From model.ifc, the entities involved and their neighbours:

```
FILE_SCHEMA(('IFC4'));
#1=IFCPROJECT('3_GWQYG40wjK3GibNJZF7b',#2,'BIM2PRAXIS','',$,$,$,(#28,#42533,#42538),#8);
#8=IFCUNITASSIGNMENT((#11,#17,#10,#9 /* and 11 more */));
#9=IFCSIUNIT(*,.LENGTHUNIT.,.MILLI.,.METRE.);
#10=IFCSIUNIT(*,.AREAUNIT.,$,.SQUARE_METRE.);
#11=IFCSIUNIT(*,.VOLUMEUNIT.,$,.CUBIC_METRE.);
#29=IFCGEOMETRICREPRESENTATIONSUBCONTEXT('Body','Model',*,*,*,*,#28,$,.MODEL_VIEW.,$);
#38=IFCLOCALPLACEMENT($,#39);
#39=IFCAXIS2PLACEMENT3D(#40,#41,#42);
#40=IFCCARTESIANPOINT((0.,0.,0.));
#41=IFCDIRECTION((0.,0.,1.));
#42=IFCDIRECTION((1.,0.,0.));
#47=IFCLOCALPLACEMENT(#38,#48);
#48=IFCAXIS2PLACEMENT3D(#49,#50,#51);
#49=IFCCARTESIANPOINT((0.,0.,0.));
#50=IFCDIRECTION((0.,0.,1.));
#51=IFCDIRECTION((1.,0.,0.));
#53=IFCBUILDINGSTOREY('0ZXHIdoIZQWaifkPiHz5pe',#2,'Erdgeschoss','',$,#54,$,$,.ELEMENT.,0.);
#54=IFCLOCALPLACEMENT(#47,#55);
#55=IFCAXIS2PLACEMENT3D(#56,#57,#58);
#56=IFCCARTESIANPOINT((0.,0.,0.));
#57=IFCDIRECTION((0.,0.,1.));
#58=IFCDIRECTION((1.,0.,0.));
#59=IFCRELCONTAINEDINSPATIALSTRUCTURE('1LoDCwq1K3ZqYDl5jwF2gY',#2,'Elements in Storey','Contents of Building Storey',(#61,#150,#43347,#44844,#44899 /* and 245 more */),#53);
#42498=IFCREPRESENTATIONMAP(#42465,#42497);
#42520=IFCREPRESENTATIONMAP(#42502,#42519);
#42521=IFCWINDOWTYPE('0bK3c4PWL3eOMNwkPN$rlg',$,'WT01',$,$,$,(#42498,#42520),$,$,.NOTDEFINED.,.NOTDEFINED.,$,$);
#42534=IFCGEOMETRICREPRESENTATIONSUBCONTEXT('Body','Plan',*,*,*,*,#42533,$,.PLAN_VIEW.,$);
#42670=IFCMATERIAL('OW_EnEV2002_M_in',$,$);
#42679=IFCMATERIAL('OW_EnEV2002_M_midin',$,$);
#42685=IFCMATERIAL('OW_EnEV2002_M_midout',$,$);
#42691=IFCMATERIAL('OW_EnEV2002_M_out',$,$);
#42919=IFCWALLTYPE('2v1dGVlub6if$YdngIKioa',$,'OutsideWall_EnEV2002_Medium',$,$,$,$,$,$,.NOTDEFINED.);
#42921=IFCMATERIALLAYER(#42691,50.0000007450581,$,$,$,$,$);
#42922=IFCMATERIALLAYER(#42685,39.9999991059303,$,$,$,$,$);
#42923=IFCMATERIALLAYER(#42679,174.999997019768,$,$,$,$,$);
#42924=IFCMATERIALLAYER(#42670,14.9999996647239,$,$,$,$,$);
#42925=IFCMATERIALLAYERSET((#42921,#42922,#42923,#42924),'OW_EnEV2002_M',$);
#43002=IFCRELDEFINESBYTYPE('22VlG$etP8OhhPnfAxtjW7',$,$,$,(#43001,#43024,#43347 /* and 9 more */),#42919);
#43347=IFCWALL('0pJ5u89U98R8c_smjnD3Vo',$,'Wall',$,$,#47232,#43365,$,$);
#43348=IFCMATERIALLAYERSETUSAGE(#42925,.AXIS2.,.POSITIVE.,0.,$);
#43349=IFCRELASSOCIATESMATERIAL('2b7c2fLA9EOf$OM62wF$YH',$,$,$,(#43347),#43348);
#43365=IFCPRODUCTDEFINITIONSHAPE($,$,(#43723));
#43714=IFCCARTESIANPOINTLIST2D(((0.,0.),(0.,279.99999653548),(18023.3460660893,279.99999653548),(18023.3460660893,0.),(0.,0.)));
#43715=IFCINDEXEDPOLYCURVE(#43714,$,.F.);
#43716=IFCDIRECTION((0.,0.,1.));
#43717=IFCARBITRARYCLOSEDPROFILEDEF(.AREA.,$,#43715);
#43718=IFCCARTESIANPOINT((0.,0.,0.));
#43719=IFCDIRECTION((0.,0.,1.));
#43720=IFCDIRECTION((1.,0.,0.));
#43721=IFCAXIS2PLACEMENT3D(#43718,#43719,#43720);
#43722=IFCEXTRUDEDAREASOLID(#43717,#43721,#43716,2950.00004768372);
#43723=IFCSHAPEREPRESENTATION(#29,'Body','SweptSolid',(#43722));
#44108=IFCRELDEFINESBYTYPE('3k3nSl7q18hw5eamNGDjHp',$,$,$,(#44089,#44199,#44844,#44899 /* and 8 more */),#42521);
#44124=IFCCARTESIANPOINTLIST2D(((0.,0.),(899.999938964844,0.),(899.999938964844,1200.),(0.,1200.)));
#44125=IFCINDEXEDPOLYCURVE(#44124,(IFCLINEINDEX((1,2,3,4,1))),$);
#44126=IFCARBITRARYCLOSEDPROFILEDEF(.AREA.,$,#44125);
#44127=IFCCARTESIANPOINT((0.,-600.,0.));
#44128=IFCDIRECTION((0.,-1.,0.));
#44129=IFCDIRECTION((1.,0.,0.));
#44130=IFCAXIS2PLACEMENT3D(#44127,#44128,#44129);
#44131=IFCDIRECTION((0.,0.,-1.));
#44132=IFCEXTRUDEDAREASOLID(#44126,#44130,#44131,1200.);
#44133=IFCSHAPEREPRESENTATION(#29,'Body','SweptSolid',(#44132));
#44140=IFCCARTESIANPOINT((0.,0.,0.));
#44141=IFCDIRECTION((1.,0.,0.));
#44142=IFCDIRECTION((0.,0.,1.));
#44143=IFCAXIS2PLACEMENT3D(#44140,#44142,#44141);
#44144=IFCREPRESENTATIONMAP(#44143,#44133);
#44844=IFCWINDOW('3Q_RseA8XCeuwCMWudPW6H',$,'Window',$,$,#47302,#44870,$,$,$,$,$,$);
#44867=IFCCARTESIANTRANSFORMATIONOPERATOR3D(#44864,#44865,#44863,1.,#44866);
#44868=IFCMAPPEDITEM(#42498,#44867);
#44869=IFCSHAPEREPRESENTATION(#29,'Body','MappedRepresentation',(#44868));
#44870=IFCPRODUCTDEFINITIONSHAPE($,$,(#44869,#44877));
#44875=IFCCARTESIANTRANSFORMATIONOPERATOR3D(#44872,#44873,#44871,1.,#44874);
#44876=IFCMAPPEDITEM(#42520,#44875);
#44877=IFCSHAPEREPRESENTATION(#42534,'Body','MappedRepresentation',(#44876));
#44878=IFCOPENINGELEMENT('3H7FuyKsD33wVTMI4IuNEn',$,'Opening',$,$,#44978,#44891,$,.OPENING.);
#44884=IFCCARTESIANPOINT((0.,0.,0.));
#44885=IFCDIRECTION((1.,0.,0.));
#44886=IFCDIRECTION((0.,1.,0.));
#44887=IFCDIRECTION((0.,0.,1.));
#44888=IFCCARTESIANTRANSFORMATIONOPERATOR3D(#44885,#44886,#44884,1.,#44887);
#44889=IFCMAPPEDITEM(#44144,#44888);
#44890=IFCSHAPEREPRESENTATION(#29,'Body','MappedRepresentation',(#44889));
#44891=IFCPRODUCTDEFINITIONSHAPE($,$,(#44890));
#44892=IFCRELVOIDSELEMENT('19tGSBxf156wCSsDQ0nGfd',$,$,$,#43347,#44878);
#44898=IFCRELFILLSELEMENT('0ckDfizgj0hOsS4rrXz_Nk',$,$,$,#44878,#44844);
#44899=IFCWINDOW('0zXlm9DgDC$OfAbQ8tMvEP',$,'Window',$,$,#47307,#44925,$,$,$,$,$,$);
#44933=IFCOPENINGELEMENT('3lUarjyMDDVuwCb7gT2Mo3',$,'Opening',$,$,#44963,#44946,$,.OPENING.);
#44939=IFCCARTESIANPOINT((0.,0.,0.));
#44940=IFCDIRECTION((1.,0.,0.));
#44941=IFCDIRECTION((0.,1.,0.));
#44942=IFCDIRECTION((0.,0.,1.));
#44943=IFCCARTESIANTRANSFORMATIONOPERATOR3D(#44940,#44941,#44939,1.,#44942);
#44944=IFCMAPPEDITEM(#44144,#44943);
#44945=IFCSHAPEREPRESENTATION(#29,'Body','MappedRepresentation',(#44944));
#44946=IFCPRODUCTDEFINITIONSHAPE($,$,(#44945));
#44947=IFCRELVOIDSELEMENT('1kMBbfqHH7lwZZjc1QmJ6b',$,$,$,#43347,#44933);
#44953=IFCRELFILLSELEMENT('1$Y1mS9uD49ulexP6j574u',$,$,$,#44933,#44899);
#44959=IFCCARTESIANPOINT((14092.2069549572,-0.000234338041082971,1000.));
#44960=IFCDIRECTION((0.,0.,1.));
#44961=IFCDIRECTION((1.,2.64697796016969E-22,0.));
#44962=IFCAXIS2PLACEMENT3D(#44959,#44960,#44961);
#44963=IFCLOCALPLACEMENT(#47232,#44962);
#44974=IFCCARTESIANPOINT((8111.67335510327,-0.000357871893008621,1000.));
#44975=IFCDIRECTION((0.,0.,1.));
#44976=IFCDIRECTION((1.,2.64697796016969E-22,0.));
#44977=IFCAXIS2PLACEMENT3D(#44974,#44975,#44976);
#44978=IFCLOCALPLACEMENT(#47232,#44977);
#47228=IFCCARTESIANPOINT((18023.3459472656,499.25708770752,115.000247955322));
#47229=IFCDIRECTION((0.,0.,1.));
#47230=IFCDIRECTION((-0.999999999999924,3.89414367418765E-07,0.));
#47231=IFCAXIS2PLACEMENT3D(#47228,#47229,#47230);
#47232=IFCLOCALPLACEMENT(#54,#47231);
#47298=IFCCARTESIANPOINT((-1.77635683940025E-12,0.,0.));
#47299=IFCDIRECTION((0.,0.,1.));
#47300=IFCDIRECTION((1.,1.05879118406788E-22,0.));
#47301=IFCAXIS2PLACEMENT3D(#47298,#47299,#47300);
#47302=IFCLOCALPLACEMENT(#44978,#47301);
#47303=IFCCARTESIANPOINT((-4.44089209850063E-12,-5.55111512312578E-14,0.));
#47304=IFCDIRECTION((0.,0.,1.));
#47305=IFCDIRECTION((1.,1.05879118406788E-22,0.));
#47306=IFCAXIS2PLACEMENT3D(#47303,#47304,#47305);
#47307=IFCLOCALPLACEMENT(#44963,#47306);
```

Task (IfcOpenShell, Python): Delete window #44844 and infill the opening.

```python
import ifcopenshell
import ifcopenshell.api.feature
import ifcopenshell.api.root
import ifcopenshell.geom
import ifcopenshell.util.shape

model = ifcopenshell.open("model.ifc")
settings = ifcopenshell.geom.settings()


def volume(element):
    """Net volume in cubic metres, openings subtracted."""
    shape = ifcopenshell.geom.create_shape(settings, element)
    return ifcopenshell.util.shape.get_volume(shape.geometry)


window = model.by_id(44844)
opening = window.FillsVoids[0].RelatingOpeningElement
wall = opening.VoidsElements[0].RelatingBuildingElement
before = volume(wall)

ifcopenshell.api.root.remove_product(model, product=window)
ifcopenshell.api.feature.remove_feature(model, feature=opening)

after = volume(wall)

print(f"wall volume {before:.3f} -> {after:.3f} m3")

model.write("model_rev.ifc")
```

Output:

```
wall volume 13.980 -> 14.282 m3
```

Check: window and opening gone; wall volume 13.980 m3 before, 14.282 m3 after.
